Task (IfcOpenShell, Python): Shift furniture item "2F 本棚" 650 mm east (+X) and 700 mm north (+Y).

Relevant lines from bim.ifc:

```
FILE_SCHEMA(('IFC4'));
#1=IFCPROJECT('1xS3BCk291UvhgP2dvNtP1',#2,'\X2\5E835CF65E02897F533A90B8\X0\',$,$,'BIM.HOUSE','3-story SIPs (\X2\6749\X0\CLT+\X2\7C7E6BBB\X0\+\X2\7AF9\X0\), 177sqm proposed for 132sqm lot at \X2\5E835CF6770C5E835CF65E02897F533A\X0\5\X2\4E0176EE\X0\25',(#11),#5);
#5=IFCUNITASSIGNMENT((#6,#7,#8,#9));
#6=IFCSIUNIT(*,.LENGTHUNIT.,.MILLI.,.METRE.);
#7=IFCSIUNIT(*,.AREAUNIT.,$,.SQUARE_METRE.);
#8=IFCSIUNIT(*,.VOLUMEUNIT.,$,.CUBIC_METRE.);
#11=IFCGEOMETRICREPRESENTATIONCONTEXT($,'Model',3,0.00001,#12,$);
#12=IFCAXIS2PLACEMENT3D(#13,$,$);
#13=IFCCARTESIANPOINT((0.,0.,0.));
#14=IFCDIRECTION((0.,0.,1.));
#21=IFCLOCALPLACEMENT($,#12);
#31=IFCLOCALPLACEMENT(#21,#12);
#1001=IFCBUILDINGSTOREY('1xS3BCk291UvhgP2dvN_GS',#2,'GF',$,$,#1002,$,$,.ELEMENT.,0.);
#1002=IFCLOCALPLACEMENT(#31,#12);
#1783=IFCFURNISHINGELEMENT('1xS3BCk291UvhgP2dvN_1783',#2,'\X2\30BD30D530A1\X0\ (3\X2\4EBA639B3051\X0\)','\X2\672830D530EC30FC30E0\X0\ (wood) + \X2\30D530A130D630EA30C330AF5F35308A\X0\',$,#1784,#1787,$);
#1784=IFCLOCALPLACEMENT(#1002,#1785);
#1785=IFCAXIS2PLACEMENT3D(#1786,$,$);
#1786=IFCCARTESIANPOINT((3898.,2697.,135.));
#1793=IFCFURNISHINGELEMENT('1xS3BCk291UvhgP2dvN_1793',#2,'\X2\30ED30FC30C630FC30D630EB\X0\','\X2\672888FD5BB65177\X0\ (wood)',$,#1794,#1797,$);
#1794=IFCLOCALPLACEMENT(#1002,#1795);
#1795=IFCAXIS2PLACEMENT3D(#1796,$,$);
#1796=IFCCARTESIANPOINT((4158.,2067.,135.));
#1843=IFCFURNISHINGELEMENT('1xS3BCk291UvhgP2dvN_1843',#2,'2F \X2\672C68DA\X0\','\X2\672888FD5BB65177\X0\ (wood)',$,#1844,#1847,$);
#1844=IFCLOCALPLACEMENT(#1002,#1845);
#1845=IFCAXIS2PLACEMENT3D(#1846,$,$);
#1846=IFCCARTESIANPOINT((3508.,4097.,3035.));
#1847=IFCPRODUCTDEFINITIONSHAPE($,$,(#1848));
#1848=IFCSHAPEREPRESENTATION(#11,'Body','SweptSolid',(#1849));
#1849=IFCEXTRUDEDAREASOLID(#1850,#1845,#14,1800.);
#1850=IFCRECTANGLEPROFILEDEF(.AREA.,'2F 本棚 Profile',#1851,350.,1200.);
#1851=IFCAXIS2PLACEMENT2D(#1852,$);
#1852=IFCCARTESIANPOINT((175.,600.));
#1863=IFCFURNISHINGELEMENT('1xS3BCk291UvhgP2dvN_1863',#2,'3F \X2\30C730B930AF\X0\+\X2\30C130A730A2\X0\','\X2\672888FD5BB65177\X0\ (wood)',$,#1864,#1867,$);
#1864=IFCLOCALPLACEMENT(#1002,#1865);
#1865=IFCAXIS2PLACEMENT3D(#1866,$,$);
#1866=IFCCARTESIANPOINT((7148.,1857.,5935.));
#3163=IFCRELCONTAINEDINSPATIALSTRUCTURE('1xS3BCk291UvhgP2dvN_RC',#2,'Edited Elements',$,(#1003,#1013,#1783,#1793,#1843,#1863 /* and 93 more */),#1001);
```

```python
import ifcopenshell
import ifcopenshell.api.geometry
import ifcopenshell.util.placement
import ifcopenshell.util.unit

model = ifcopenshell.open("bim.ifc")
unit_scale = ifcopenshell.util.unit.calculate_unit_scale(model)

item = model.by_guid("1xS3BCk291UvhgP2dvN_1843")
matrix = ifcopenshell.util.placement.get_local_placement(item.ObjectPlacement)
matrix[0, 3] += 0.65 / unit_scale
matrix[1, 3] += 0.7 / unit_scale
ifcopenshell.api.geometry.edit_object_placement(model, product=item, matrix=matrix, is_si=False)

print(ifcopenshell.util.placement.get_local_placement(item.ObjectPlacement).round(3) + 0.0)

model.write("bim_edited.ifc")
```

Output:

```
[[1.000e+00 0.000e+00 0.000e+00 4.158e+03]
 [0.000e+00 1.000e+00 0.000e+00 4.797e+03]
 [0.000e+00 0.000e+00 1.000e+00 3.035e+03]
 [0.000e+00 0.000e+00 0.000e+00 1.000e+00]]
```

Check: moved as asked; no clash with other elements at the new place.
